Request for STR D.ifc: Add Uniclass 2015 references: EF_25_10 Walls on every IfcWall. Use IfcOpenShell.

First a look at what the model holds.

```python
import ifcopenshell

model = ifcopenshell.open("STR D.ifc")
print(model.schema)
print("classifications:", [c.Name for c in model.by_type("IfcClassification")])
for ifc_class in ("IfcDoor", "IfcRoof", "IfcStair", "IfcWall", "IfcWindow"):
    print(ifc_class, len(model.by_type(ifc_class)))
```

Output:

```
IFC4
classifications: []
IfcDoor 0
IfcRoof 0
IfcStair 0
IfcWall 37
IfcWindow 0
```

```python
import ifcopenshell
import ifcopenshell.api.classification

model = ifcopenshell.open("STR D.ifc")

system = ifcopenshell.api.classification.add_classification(model, classification="Uniclass 2015")

codes = {
    "IfcWall": ("EF_25_10", "Walls"),
}
for ifc_class, (code, name) in codes.items():
    products = model.by_type(ifc_class)
    ifcopenshell.api.classification.add_reference(
        model, products=products, classification=system, identification=code, name=name
    )
    print(code, len(products))

model.write("STR D_updated.ifc")
```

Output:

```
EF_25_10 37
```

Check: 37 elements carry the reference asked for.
